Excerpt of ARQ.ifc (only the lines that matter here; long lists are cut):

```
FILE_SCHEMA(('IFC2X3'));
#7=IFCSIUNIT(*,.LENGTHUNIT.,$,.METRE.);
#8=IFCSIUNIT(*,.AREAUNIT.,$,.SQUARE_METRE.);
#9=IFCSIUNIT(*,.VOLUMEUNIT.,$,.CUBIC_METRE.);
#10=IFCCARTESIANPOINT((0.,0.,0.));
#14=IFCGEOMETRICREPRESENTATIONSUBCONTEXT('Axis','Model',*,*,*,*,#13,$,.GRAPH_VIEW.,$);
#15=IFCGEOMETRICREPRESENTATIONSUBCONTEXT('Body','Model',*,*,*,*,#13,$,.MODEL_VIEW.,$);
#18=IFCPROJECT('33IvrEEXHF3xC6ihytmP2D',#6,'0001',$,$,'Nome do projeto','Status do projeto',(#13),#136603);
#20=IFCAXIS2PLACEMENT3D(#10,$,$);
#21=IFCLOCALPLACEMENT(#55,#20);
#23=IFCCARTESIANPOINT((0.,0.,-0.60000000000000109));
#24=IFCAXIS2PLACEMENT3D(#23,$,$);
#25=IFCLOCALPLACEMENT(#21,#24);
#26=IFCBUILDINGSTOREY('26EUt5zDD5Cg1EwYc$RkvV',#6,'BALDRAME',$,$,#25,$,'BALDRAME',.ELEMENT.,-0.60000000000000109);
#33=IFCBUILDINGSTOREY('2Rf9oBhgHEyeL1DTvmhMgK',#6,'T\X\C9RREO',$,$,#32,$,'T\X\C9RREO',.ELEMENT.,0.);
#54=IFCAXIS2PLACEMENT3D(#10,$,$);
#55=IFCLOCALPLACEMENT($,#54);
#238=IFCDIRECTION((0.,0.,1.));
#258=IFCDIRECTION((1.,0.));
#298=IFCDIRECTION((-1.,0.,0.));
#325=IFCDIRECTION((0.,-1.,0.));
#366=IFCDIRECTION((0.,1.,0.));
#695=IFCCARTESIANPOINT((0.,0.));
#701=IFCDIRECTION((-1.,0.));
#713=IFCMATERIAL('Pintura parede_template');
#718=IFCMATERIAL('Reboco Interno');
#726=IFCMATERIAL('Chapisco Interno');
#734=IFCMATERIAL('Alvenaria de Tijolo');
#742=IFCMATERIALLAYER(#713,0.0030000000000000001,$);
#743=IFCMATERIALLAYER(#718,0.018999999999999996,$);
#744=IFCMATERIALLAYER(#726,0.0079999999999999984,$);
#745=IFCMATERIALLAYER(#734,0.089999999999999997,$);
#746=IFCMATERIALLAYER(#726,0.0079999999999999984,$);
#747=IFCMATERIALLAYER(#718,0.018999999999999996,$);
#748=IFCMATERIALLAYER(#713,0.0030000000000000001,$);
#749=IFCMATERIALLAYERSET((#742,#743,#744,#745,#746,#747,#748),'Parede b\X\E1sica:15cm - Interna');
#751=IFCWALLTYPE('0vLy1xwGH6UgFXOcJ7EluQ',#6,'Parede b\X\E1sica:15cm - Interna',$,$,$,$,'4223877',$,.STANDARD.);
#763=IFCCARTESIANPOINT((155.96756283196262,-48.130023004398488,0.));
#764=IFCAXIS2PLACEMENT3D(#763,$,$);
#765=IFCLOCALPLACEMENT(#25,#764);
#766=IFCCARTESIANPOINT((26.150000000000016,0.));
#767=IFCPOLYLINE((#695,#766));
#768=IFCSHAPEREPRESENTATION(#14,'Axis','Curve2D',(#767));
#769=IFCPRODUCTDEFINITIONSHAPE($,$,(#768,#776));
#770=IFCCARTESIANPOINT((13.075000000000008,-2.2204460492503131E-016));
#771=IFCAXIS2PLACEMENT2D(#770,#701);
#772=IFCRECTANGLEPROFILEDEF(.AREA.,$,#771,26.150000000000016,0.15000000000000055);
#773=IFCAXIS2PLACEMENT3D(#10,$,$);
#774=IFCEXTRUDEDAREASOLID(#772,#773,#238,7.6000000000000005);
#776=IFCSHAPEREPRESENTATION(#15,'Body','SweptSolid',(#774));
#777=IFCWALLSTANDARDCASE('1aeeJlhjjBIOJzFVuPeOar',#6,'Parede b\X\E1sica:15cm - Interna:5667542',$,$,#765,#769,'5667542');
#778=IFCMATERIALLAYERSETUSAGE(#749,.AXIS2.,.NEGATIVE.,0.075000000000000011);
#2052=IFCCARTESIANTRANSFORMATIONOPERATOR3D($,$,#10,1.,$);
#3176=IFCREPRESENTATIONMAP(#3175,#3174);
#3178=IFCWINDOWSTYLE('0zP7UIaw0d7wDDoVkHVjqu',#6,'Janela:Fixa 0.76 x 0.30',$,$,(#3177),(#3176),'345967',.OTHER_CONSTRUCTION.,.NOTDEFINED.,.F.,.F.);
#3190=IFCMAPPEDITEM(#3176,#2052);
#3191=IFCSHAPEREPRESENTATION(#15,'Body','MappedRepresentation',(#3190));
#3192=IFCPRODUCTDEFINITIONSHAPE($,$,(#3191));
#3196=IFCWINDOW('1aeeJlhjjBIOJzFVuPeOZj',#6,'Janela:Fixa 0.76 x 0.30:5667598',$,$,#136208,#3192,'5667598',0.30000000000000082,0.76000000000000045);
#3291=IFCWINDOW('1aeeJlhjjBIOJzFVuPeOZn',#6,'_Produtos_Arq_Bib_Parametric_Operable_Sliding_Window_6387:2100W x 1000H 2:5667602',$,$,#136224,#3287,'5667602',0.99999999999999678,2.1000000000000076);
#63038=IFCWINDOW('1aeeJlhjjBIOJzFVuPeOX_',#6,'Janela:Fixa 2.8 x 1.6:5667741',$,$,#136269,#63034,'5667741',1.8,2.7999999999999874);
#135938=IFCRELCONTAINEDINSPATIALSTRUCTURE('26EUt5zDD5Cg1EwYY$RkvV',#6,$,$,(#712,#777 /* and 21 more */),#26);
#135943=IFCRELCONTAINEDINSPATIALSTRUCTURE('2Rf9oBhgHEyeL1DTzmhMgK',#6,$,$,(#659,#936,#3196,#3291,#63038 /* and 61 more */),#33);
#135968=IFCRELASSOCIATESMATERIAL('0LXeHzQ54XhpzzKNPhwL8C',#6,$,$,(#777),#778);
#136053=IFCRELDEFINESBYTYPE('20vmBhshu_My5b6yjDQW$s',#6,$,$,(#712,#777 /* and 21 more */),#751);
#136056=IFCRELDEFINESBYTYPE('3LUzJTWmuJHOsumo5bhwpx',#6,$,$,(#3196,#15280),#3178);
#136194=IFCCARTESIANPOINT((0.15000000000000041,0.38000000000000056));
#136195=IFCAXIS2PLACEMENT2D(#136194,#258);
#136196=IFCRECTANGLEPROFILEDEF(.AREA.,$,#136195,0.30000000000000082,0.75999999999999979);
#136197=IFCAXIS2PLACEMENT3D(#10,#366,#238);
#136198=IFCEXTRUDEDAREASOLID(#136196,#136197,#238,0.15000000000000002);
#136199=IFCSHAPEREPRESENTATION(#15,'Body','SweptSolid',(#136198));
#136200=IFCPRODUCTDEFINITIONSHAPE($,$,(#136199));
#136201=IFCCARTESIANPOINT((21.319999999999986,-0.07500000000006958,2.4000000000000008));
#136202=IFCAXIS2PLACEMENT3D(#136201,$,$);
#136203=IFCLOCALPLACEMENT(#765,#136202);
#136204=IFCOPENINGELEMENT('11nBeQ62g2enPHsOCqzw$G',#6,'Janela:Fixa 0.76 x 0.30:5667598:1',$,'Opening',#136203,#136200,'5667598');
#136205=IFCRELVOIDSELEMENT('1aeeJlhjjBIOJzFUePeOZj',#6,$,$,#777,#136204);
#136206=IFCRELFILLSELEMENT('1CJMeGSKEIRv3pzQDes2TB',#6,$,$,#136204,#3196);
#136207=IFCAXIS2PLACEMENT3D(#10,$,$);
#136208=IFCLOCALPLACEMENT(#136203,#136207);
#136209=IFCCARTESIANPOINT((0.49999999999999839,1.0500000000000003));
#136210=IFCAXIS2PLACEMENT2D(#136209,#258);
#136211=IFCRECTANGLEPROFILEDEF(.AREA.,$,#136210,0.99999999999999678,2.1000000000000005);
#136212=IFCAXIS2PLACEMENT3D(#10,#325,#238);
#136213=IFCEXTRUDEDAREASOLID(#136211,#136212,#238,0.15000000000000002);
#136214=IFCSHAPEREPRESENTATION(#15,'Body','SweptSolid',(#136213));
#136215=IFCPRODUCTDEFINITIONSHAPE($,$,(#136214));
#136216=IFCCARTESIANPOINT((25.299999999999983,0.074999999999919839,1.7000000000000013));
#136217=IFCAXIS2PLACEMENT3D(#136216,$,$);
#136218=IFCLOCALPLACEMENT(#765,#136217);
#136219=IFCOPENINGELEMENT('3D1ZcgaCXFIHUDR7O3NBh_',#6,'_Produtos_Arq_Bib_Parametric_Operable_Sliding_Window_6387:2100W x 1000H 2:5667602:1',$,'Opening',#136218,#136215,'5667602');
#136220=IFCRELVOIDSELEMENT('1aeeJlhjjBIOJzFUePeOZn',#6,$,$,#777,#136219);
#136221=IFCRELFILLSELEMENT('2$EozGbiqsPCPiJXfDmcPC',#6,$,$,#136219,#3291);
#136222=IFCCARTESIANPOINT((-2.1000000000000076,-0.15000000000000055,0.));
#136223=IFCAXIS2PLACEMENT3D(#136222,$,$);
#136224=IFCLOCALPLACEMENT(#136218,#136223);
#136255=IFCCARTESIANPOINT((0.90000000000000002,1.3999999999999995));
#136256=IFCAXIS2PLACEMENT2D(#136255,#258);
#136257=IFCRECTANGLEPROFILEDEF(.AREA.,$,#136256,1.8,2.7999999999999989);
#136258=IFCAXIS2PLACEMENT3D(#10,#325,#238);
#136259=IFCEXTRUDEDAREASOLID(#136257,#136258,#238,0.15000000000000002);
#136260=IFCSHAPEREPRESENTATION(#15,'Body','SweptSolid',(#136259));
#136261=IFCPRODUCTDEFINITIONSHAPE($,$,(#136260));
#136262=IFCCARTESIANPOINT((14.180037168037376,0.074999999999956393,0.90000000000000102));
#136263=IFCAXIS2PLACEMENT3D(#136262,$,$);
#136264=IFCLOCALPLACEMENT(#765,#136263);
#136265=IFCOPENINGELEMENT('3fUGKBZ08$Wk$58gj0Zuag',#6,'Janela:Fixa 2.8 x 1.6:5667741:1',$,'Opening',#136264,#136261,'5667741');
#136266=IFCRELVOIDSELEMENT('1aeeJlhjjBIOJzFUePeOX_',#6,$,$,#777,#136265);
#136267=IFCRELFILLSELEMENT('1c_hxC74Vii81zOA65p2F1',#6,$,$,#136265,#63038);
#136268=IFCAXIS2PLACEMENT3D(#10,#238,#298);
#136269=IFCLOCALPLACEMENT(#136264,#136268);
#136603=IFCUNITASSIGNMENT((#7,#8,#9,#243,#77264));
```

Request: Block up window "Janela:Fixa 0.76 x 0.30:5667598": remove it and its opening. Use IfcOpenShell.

```python
import ifcopenshell
import ifcopenshell.api.feature
import ifcopenshell.api.root
import ifcopenshell.geom
import ifcopenshell.util.shape

model = ifcopenshell.open("ARQ.ifc")
settings = ifcopenshell.geom.settings()


def volume(element):
    """Net volume in cubic metres, openings subtracted."""
    shape = ifcopenshell.geom.create_shape(settings, element)
    return ifcopenshell.util.shape.get_volume(shape.geometry)


window = model.by_guid("1aeeJlhjjBIOJzFVuPeOZj")
opening = window.FillsVoids[0].RelatingOpeningElement
wall = opening.VoidsElements[0].RelatingBuildingElement
before = volume(wall)

ifcopenshell.api.root.remove_product(model, product=window)
ifcopenshell.api.feature.remove_feature(model, feature=opening)

after = volume(wall)

print(f"wall volume {before:.3f} -> {after:.3f} m3")

model.write("ARQ_rev.ifc")
```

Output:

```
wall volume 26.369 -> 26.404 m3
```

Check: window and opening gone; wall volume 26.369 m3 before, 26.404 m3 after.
